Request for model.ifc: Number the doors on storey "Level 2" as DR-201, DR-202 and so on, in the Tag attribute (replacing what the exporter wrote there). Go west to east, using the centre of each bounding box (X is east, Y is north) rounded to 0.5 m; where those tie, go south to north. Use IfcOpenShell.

First a look at what the model holds.

```python
import ifcopenshell
import ifcopenshell.util.element
import ifcopenshell.util.placement

model = ifcopenshell.open("model.ifc")
print(model.schema)
storey = next(s for s in model.by_type("IfcBuildingStorey") if s.Name == "Level 2")
doors = [e for e in ifcopenshell.util.element.get_decomposition(storey) if e.is_a("IfcDoor")]
for e in sorted(doors, key=lambda e: e.id()):
    origin = ifcopenshell.util.placement.get_local_placement(e.ObjectPlacement)[:3, 3]
    print(e.id(), e.Tag, e.Name, origin.round(2) + 0.0, sep=" | ")
```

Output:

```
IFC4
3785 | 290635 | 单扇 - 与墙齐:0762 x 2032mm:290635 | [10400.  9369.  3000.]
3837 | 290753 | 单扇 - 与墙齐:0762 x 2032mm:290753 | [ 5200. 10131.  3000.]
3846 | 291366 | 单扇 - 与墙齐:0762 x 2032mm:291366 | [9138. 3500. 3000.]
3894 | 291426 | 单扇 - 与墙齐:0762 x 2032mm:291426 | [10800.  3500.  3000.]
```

```python
import ifcopenshell
import ifcopenshell.geom
import ifcopenshell.util.element
import ifcopenshell.util.shape

model = ifcopenshell.open("model.ifc")
settings = ifcopenshell.geom.settings()
settings.set("use-world-coords", True)


def centre(element):
    shape = ifcopenshell.geom.create_shape(settings, element)
    return ifcopenshell.util.shape.get_bbox_centroid(shape.geometry)


storey = next(s for s in model.by_type("IfcBuildingStorey") if s.Name == "Level 2")
doors = [e for e in ifcopenshell.util.element.get_decomposition(storey) if e.is_a("IfcDoor")]

# Insertion points can sit at a corner or the storey origin, so sort by the geometry (in metres).
centres = {e: centre(e) for e in doors}
doors.sort(key=lambda e: (round(centres[e][0] / 0.5), centres[e][1]))

for i, e in enumerate(doors, start=1):
    number = f"DR-2{i:02d}"
    e.Tag = number
    print(e.id(), number)

model.write("model_v2.ifc")
```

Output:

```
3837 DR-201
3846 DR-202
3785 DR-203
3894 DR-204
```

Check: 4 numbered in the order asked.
